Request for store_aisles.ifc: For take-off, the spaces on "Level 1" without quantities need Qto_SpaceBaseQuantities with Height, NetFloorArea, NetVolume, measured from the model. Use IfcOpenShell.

First a look at what the model holds.

```python
import ifcopenshell
import ifcopenshell.util.element
import ifcopenshell.util.unit

model = ifcopenshell.open("store_aisles.ifc")
print(model.schema)
for unit_type in ("LENGTHUNIT", "AREAUNIT", "VOLUMEUNIT"):
    print(unit_type, ifcopenshell.util.unit.calculate_unit_scale(model, unit_type))
storey = next(s for s in model.by_type("IfcBuildingStorey") if s.Name == "Level 1")
spaces = [e for e in ifcopenshell.util.element.get_decomposition(storey) if e.is_a("IfcSpace")]
for e in sorted(spaces, key=lambda e: e.id()):
    print(e.id(), e.is_a(), e.Name, list(ifcopenshell.util.element.get_psets(e, qtos_only=True)), sep=" | ")
```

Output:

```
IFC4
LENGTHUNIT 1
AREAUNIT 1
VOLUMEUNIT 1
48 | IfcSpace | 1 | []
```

```python
import ifcopenshell
import ifcopenshell.api.pset
import ifcopenshell.geom
import ifcopenshell.util.element
import ifcopenshell.util.shape
import ifcopenshell.util.unit

model = ifcopenshell.open("store_aisles.ifc")
unit_scale = ifcopenshell.util.unit.calculate_unit_scale(model)
area_scale = ifcopenshell.util.unit.calculate_unit_scale(model, "AREAUNIT")
volume_scale = ifcopenshell.util.unit.calculate_unit_scale(model, "VOLUMEUNIT")
settings = ifcopenshell.geom.settings()

storey = next(s for s in model.by_type("IfcBuildingStorey") if s.Name == "Level 1")
spaces = [e for e in ifcopenshell.util.element.get_decomposition(storey) if e.is_a("IfcSpace")]

for e in sorted(spaces, key=lambda e: e.id()):
    if ifcopenshell.util.element.get_psets(e, qtos_only=True, should_inherit=False):
        continue
    # Geometry comes back in metres, in the element's own axes.
    shape = ifcopenshell.geom.create_shape(settings, e)
    values = {
        "Height": ifcopenshell.util.shape.get_z(shape.geometry) / unit_scale,
        "NetFloorArea": ifcopenshell.util.shape.get_footprint_area(shape.geometry) / area_scale,
        "NetVolume": ifcopenshell.util.shape.get_volume(shape.geometry) / volume_scale,
    }
    qto = ifcopenshell.api.pset.add_qto(model, product=e, name="Qto_SpaceBaseQuantities")
    ifcopenshell.api.pset.edit_qto(model, qto=qto, properties=values)
    print(e.id(), {k: round(v, 3) for k, v in values.items()})

model.write("store_aisles_v2.ifc")
```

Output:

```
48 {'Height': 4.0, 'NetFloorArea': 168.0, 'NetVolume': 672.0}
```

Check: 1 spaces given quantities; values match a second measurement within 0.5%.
